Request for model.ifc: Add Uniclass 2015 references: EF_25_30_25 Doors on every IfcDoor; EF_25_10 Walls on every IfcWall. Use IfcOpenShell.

First a look at what the model holds.

```python
import ifcopenshell

model = ifcopenshell.open("model.ifc")
print(model.schema)
print("classifications:", [c.Name for c in model.by_type("IfcClassification")])
for ifc_class in ("IfcDoor", "IfcRoof", "IfcStair", "IfcWall", "IfcWindow"):
    print(ifc_class, len(model.by_type(ifc_class)))
```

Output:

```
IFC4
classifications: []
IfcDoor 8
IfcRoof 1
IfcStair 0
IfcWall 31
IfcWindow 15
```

```python
import ifcopenshell
import ifcopenshell.api.classification

model = ifcopenshell.open("model.ifc")

system = ifcopenshell.api.classification.add_classification(model, classification="Uniclass 2015")

codes = {
    "IfcDoor": ("EF_25_30_25", "Doors"),
    "IfcWall": ("EF_25_10", "Walls"),
}
for ifc_class, (code, name) in codes.items():
    products = model.by_type(ifc_class)
    ifcopenshell.api.classification.add_reference(
        model, products=products, classification=system, identification=code, name=name
    )
    print(code, len(products))

model.write("model_rev.ifc")
```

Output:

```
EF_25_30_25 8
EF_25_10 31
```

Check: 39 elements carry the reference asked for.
